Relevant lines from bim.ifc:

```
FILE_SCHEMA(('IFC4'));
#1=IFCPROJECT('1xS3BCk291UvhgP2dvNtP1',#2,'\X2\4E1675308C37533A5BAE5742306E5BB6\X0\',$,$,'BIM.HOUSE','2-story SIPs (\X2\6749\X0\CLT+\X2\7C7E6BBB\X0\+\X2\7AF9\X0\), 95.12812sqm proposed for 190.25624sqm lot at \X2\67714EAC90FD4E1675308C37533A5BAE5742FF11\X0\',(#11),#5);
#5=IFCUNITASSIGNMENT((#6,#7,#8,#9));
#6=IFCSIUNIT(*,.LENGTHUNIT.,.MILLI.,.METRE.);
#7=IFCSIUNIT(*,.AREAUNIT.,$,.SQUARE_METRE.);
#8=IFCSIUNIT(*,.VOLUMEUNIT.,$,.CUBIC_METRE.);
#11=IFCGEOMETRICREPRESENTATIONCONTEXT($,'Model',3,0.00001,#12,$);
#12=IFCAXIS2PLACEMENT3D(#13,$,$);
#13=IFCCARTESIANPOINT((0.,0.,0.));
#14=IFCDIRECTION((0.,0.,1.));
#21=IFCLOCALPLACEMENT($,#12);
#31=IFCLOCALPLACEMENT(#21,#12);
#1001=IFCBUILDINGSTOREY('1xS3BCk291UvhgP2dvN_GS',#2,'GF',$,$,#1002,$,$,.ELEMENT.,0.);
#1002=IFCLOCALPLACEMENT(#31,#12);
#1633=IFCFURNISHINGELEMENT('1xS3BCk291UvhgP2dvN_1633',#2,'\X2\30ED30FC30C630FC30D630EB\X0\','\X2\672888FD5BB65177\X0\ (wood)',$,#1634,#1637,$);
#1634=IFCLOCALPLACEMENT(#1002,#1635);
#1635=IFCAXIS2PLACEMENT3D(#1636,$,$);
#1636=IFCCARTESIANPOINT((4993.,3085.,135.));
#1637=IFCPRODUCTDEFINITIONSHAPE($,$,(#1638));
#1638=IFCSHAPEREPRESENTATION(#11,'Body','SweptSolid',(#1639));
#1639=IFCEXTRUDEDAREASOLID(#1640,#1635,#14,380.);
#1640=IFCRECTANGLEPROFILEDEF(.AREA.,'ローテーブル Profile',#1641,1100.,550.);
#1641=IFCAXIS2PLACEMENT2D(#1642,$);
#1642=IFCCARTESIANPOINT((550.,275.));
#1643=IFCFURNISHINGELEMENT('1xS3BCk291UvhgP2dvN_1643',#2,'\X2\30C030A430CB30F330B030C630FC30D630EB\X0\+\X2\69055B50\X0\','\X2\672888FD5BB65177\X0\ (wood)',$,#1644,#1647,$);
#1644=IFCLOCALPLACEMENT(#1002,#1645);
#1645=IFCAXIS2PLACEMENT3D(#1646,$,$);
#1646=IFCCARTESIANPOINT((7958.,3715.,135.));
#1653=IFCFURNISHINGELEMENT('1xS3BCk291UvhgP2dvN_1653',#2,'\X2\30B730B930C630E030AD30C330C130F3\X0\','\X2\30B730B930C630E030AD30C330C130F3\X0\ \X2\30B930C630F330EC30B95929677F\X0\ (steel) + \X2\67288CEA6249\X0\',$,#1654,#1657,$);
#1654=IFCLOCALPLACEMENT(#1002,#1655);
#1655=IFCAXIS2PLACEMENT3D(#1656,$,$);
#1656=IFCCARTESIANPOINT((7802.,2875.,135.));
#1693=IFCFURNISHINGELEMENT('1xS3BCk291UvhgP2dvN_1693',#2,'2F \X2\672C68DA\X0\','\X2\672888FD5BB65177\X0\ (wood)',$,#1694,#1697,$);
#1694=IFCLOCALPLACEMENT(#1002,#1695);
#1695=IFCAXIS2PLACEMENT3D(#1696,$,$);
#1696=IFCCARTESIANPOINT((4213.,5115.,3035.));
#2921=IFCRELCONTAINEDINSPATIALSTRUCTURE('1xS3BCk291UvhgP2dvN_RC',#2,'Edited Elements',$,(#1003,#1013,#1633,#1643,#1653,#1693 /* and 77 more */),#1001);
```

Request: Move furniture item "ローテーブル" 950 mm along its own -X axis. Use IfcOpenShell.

```python
import ifcopenshell
import ifcopenshell.api.geometry
import ifcopenshell.util.placement
import ifcopenshell.util.unit

model = ifcopenshell.open("bim.ifc")
unit_scale = ifcopenshell.util.unit.calculate_unit_scale(model)

item = model.by_id(1633)
matrix = ifcopenshell.util.placement.get_local_placement(item.ObjectPlacement)
matrix[:3, 3] -= matrix[:3, 0] * 0.95 / unit_scale
ifcopenshell.api.geometry.edit_object_placement(model, product=item, matrix=matrix, is_si=False)

print(ifcopenshell.util.placement.get_local_placement(item.ObjectPlacement).round(3) + 0.0)

model.write("bim-out.ifc")
```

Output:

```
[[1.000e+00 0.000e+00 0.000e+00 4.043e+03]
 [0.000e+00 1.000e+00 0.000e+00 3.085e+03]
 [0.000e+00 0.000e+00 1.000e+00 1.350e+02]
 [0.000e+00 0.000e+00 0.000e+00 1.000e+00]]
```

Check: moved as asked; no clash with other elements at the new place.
